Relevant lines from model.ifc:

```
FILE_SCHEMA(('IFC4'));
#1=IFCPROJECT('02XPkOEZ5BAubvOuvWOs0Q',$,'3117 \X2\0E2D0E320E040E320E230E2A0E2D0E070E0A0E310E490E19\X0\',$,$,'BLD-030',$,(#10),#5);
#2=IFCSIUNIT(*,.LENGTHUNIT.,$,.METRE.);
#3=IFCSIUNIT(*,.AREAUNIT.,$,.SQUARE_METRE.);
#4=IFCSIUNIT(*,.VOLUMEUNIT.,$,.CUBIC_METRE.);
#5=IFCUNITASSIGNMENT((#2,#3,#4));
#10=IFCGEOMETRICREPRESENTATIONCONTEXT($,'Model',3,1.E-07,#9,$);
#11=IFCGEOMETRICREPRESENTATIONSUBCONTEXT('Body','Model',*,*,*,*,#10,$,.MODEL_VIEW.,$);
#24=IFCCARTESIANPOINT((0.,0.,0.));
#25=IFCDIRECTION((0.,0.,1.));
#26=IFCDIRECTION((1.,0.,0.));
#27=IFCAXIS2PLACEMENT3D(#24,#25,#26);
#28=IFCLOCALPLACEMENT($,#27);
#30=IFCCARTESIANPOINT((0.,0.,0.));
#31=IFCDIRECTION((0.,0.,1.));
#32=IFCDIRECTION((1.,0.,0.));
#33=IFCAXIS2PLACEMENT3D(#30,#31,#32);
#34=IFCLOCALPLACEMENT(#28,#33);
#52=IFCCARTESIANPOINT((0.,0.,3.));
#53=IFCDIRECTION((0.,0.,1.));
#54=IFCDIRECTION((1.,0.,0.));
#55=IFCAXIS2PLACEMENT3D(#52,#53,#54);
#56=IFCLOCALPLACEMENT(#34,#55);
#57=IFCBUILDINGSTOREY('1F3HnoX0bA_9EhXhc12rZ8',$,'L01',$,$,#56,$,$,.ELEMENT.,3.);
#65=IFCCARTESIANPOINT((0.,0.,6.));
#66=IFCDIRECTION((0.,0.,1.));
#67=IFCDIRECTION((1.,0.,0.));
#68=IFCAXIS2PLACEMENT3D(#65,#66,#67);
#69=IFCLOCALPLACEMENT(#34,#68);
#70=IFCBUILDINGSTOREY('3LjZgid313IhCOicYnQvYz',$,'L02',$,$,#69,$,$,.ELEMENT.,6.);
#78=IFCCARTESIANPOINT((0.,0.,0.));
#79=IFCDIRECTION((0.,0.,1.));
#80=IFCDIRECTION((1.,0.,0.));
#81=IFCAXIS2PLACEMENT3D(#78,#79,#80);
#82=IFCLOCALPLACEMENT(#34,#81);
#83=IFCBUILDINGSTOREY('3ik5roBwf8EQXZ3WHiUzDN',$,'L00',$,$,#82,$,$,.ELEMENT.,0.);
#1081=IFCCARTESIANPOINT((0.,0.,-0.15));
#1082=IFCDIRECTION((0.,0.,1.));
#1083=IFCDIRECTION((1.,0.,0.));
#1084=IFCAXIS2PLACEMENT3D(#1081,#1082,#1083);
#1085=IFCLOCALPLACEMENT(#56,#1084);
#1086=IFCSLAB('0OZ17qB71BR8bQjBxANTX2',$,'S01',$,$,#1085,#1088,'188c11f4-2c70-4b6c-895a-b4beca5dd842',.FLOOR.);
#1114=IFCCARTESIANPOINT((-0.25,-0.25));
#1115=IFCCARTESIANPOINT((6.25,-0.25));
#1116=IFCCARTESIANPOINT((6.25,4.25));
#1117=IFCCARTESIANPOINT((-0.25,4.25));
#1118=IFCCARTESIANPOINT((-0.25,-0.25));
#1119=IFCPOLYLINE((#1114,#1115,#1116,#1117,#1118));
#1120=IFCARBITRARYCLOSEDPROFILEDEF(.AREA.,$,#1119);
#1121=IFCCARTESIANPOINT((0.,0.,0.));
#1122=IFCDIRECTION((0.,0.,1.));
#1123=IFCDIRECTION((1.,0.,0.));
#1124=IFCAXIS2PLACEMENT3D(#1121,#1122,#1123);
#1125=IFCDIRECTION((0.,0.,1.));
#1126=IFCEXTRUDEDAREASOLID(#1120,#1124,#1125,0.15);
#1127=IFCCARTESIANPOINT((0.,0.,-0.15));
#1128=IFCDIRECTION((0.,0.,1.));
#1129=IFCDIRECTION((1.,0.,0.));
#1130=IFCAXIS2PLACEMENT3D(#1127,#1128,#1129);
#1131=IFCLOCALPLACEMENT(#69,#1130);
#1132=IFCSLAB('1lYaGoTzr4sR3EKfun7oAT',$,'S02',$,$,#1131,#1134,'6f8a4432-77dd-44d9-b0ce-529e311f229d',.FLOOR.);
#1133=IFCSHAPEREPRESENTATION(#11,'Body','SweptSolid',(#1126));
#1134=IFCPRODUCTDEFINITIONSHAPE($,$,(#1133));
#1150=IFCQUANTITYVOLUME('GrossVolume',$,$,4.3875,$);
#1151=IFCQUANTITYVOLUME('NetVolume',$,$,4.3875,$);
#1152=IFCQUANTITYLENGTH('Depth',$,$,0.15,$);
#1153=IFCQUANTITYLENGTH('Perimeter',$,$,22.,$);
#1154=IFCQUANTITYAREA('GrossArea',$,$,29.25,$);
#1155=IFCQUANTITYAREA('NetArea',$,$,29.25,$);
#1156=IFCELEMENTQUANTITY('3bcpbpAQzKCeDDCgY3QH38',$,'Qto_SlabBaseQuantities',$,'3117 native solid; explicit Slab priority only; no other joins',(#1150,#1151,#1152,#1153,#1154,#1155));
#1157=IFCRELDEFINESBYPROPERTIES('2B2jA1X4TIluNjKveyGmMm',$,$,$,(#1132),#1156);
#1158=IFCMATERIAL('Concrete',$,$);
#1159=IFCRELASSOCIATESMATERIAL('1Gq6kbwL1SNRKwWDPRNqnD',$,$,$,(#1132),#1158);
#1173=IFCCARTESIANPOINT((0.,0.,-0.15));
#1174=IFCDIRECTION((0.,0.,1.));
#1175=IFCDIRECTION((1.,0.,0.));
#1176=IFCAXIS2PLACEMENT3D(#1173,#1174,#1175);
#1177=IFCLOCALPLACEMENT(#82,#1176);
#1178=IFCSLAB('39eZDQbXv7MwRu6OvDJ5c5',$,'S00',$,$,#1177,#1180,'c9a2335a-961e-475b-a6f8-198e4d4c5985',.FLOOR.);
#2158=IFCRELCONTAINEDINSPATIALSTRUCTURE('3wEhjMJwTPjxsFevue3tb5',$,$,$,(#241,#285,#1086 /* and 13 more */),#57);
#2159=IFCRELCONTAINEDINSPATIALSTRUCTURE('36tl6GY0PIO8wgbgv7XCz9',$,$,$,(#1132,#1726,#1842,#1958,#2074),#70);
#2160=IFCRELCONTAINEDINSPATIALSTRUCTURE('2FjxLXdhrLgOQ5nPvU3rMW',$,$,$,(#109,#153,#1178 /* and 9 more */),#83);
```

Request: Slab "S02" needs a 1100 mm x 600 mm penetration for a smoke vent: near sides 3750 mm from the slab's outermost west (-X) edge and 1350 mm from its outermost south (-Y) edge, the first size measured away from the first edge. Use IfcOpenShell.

```python
import numpy as np
import ifcopenshell
import ifcopenshell.api.feature
import ifcopenshell.api.geometry
import ifcopenshell.api.pset
import ifcopenshell.api.root
import ifcopenshell.geom
import ifcopenshell.util.element
import ifcopenshell.util.placement
import ifcopenshell.util.representation
import ifcopenshell.util.shape
import ifcopenshell.util.unit

model = ifcopenshell.open("model.ifc")
unit_scale = ifcopenshell.util.unit.calculate_unit_scale(model)
area_scale = ifcopenshell.util.unit.calculate_unit_scale(model, "AREAUNIT")
volume_scale = ifcopenshell.util.unit.calculate_unit_scale(model, "VOLUMEUNIT")
settings = ifcopenshell.geom.settings()


def volume(element):
    """Net volume in cubic metres, openings subtracted."""
    shape = ifcopenshell.geom.create_shape(settings, element)
    return ifcopenshell.util.shape.get_volume(shape.geometry)


slab = model.by_guid("1lYaGoTzr4sR3EKfun7oAT")
before = volume(slab)

# Extent in the slab's own axes, in metres. The edges named are its -X and -Y sides.
slab_shape = ifcopenshell.geom.create_shape(settings, slab)
vertices = ifcopenshell.util.shape.get_vertices(slab_shape.geometry)
x_min, y_min, bottom = vertices.min(axis=0)
top = vertices[:, 2].max()

opening = ifcopenshell.api.root.create_entity(model, ifc_class="IfcOpeningElement", name="Smoke vent opening", predefined_type="OPENING")
context = ifcopenshell.util.representation.get_context(model, "Model", "Body", "MODEL_VIEW")
width, depth = 1.1, 0.6
outline = [(0.0, 0.0), (width, 0.0), (width, depth), (0.0, depth), (0.0, 0.0)]
# Overshoot both faces by 50 mm so the cut is clean.
shape = ifcopenshell.api.geometry.add_slab_representation(
    model, context=context, depth=top - bottom + 0.1, polyline=outline
)
ifcopenshell.api.geometry.assign_representation(model, product=opening, representation=shape)

matrix = ifcopenshell.util.placement.get_local_placement(slab.ObjectPlacement)
matrix[:, 3] = matrix @ np.append(np.array([x_min + 3.75, y_min + 1.35, bottom - 0.05]) / unit_scale, 1.0)
ifcopenshell.api.geometry.edit_object_placement(model, product=opening, matrix=matrix, is_si=False)
ifcopenshell.api.feature.add_feature(model, feature=opening, element=slab)

after = volume(slab)

# Update the slab's stored quantities.
qto = model.by_id(ifcopenshell.util.element.get_pset(slab, "Qto_SlabBaseQuantities", should_inherit=False)["id"])
ifcopenshell.api.pset.edit_qto(model, qto=qto, properties={
    "NetVolume": after / volume_scale,
    "NetArea": after / (top - bottom) / area_scale,
})

print(f"slab volume {before:.3f} -> {after:.3f} m3")

model.write("model_v2.ifc")
```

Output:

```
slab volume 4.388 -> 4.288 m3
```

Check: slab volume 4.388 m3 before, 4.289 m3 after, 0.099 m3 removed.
